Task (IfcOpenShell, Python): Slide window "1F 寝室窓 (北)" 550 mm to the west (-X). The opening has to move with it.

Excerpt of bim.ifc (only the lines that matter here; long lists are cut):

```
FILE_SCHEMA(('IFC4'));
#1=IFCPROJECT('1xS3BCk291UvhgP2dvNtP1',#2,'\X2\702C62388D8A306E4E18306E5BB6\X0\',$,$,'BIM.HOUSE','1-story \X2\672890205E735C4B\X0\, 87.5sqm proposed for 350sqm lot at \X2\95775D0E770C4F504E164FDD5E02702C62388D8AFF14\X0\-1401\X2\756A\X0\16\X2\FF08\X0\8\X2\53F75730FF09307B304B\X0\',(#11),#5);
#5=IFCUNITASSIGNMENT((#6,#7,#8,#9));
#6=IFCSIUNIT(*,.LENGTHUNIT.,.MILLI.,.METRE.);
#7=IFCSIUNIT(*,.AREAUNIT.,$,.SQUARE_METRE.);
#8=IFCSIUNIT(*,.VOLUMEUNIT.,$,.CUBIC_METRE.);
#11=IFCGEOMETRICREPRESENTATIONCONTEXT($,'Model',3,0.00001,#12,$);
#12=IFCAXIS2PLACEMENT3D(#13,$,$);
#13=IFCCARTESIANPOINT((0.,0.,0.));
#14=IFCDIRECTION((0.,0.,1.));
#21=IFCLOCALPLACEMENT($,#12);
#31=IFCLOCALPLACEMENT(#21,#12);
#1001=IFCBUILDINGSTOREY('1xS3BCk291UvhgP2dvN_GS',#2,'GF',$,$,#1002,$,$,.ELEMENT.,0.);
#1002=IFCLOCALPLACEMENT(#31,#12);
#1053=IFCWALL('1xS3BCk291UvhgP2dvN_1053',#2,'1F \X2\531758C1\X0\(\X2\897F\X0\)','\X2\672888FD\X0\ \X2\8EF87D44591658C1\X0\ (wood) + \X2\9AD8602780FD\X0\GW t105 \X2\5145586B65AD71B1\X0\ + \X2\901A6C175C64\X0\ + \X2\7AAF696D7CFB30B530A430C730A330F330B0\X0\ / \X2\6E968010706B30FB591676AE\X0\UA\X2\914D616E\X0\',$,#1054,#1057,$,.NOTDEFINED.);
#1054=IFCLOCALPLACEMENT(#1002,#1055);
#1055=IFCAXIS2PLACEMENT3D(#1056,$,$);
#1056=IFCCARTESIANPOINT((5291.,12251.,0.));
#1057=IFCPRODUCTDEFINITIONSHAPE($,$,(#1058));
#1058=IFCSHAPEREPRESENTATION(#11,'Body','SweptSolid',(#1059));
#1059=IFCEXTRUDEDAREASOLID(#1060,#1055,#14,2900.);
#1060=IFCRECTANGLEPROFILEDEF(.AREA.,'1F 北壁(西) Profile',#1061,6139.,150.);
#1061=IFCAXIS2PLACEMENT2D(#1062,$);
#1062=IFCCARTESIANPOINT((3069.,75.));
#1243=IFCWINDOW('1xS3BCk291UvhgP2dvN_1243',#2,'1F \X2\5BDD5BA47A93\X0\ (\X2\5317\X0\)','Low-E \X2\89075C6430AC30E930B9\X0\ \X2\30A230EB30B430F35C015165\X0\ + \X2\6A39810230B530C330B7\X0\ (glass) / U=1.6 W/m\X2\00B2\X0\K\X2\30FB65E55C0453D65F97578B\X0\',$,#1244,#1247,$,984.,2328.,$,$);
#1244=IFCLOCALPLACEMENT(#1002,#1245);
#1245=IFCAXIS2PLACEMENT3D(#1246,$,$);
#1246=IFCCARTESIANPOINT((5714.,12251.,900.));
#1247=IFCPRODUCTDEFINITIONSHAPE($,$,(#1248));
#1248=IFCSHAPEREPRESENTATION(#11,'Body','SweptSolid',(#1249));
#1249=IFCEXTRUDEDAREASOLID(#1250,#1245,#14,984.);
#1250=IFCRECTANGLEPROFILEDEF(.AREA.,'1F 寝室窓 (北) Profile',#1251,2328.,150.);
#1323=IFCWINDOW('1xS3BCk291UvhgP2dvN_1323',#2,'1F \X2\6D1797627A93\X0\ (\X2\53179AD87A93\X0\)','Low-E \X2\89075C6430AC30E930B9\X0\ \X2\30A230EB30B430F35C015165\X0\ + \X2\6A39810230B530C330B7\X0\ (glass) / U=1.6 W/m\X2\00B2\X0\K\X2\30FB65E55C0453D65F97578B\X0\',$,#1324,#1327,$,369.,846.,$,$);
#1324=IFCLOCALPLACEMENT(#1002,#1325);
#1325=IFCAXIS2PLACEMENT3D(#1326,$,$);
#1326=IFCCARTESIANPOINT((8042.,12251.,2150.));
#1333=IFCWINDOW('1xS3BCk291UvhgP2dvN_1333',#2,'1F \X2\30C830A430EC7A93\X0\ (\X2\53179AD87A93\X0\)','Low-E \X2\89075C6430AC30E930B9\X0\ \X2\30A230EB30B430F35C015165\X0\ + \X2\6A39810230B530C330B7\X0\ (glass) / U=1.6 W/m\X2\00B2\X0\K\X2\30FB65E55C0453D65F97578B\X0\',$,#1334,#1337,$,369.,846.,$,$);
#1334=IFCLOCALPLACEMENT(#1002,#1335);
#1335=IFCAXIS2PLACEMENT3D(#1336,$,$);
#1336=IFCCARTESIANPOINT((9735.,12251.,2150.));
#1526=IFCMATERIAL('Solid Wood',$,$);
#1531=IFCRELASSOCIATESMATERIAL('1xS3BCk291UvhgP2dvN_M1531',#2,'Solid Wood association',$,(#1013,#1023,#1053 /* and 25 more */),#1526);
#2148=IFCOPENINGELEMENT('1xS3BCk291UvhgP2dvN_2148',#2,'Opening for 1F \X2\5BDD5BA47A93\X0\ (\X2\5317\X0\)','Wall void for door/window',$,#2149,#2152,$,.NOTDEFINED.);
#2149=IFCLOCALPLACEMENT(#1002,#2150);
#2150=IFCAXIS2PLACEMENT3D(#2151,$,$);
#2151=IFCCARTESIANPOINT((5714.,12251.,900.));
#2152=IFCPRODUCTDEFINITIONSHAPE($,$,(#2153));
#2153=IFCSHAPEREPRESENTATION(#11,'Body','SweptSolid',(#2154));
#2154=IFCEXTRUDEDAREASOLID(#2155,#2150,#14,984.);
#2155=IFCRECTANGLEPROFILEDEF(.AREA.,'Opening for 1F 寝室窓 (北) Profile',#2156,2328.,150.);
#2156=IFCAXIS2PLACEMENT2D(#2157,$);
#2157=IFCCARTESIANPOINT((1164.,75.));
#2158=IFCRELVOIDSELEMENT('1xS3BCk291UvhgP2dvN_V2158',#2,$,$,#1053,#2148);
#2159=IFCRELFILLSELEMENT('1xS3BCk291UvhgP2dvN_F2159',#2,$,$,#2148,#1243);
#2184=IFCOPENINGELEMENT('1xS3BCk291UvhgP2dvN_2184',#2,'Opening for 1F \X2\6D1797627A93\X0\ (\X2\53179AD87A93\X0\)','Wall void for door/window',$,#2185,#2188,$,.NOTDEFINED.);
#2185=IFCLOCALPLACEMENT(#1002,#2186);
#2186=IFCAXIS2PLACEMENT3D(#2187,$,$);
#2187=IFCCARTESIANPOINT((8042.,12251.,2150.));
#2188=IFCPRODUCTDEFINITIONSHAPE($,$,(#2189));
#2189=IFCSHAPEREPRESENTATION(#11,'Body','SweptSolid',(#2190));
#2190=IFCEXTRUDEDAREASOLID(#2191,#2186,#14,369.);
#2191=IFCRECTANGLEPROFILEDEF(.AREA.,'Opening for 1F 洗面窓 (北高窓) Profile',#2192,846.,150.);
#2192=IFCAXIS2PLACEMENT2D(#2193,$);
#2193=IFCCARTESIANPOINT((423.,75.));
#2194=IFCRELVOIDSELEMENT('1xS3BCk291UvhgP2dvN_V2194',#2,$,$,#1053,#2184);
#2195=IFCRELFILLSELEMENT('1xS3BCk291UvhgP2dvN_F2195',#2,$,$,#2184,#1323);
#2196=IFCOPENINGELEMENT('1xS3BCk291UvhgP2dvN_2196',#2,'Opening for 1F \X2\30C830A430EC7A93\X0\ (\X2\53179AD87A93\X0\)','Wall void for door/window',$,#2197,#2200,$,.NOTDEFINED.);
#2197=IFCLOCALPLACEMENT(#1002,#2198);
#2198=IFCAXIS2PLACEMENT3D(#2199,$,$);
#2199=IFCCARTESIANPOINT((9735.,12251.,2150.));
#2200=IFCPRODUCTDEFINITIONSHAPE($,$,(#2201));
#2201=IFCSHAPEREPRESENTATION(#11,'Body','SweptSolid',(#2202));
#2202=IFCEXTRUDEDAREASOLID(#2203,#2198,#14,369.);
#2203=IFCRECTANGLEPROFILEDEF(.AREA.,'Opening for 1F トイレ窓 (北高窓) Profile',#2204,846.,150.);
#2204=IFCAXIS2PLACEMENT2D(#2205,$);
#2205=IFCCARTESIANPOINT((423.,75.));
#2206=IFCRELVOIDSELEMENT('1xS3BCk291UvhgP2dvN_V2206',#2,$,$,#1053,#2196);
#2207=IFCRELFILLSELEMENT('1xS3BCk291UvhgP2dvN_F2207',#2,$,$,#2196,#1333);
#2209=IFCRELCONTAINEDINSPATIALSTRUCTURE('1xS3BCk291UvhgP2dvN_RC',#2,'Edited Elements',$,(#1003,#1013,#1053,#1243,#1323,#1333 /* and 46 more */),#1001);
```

```python
import ifcopenshell
import ifcopenshell.api.geometry
import ifcopenshell.util.placement
import ifcopenshell.util.unit

model = ifcopenshell.open("bim.ifc")
unit_scale = ifcopenshell.util.unit.calculate_unit_scale(model)

window = model.by_id(1243)
opening = window.FillsVoids[0].RelatingOpeningElement
wall = opening.VoidsElements[0].RelatingBuildingElement

wall_matrix = ifcopenshell.util.placement.get_local_placement(wall.ObjectPlacement)
shift = wall_matrix[:3, 0] * -0.55 / unit_scale
before = ifcopenshell.util.placement.get_local_placement(window.ObjectPlacement)[:3, 3].copy()

# The window is not placed relative to its opening, so move both.
for product in (opening, window):
    matrix = ifcopenshell.util.placement.get_local_placement(product.ObjectPlacement)
    matrix[:3, 3] += shift
    ifcopenshell.api.geometry.edit_object_placement(model, product=product, matrix=matrix, is_si=False)

after = ifcopenshell.util.placement.get_local_placement(window.ObjectPlacement)[:3, 3]
print("window moved by", (after - before).round(3) + 0.0)

model.write("bim_updated.ifc")
```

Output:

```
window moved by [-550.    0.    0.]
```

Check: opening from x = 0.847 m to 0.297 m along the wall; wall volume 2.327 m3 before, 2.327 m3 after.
